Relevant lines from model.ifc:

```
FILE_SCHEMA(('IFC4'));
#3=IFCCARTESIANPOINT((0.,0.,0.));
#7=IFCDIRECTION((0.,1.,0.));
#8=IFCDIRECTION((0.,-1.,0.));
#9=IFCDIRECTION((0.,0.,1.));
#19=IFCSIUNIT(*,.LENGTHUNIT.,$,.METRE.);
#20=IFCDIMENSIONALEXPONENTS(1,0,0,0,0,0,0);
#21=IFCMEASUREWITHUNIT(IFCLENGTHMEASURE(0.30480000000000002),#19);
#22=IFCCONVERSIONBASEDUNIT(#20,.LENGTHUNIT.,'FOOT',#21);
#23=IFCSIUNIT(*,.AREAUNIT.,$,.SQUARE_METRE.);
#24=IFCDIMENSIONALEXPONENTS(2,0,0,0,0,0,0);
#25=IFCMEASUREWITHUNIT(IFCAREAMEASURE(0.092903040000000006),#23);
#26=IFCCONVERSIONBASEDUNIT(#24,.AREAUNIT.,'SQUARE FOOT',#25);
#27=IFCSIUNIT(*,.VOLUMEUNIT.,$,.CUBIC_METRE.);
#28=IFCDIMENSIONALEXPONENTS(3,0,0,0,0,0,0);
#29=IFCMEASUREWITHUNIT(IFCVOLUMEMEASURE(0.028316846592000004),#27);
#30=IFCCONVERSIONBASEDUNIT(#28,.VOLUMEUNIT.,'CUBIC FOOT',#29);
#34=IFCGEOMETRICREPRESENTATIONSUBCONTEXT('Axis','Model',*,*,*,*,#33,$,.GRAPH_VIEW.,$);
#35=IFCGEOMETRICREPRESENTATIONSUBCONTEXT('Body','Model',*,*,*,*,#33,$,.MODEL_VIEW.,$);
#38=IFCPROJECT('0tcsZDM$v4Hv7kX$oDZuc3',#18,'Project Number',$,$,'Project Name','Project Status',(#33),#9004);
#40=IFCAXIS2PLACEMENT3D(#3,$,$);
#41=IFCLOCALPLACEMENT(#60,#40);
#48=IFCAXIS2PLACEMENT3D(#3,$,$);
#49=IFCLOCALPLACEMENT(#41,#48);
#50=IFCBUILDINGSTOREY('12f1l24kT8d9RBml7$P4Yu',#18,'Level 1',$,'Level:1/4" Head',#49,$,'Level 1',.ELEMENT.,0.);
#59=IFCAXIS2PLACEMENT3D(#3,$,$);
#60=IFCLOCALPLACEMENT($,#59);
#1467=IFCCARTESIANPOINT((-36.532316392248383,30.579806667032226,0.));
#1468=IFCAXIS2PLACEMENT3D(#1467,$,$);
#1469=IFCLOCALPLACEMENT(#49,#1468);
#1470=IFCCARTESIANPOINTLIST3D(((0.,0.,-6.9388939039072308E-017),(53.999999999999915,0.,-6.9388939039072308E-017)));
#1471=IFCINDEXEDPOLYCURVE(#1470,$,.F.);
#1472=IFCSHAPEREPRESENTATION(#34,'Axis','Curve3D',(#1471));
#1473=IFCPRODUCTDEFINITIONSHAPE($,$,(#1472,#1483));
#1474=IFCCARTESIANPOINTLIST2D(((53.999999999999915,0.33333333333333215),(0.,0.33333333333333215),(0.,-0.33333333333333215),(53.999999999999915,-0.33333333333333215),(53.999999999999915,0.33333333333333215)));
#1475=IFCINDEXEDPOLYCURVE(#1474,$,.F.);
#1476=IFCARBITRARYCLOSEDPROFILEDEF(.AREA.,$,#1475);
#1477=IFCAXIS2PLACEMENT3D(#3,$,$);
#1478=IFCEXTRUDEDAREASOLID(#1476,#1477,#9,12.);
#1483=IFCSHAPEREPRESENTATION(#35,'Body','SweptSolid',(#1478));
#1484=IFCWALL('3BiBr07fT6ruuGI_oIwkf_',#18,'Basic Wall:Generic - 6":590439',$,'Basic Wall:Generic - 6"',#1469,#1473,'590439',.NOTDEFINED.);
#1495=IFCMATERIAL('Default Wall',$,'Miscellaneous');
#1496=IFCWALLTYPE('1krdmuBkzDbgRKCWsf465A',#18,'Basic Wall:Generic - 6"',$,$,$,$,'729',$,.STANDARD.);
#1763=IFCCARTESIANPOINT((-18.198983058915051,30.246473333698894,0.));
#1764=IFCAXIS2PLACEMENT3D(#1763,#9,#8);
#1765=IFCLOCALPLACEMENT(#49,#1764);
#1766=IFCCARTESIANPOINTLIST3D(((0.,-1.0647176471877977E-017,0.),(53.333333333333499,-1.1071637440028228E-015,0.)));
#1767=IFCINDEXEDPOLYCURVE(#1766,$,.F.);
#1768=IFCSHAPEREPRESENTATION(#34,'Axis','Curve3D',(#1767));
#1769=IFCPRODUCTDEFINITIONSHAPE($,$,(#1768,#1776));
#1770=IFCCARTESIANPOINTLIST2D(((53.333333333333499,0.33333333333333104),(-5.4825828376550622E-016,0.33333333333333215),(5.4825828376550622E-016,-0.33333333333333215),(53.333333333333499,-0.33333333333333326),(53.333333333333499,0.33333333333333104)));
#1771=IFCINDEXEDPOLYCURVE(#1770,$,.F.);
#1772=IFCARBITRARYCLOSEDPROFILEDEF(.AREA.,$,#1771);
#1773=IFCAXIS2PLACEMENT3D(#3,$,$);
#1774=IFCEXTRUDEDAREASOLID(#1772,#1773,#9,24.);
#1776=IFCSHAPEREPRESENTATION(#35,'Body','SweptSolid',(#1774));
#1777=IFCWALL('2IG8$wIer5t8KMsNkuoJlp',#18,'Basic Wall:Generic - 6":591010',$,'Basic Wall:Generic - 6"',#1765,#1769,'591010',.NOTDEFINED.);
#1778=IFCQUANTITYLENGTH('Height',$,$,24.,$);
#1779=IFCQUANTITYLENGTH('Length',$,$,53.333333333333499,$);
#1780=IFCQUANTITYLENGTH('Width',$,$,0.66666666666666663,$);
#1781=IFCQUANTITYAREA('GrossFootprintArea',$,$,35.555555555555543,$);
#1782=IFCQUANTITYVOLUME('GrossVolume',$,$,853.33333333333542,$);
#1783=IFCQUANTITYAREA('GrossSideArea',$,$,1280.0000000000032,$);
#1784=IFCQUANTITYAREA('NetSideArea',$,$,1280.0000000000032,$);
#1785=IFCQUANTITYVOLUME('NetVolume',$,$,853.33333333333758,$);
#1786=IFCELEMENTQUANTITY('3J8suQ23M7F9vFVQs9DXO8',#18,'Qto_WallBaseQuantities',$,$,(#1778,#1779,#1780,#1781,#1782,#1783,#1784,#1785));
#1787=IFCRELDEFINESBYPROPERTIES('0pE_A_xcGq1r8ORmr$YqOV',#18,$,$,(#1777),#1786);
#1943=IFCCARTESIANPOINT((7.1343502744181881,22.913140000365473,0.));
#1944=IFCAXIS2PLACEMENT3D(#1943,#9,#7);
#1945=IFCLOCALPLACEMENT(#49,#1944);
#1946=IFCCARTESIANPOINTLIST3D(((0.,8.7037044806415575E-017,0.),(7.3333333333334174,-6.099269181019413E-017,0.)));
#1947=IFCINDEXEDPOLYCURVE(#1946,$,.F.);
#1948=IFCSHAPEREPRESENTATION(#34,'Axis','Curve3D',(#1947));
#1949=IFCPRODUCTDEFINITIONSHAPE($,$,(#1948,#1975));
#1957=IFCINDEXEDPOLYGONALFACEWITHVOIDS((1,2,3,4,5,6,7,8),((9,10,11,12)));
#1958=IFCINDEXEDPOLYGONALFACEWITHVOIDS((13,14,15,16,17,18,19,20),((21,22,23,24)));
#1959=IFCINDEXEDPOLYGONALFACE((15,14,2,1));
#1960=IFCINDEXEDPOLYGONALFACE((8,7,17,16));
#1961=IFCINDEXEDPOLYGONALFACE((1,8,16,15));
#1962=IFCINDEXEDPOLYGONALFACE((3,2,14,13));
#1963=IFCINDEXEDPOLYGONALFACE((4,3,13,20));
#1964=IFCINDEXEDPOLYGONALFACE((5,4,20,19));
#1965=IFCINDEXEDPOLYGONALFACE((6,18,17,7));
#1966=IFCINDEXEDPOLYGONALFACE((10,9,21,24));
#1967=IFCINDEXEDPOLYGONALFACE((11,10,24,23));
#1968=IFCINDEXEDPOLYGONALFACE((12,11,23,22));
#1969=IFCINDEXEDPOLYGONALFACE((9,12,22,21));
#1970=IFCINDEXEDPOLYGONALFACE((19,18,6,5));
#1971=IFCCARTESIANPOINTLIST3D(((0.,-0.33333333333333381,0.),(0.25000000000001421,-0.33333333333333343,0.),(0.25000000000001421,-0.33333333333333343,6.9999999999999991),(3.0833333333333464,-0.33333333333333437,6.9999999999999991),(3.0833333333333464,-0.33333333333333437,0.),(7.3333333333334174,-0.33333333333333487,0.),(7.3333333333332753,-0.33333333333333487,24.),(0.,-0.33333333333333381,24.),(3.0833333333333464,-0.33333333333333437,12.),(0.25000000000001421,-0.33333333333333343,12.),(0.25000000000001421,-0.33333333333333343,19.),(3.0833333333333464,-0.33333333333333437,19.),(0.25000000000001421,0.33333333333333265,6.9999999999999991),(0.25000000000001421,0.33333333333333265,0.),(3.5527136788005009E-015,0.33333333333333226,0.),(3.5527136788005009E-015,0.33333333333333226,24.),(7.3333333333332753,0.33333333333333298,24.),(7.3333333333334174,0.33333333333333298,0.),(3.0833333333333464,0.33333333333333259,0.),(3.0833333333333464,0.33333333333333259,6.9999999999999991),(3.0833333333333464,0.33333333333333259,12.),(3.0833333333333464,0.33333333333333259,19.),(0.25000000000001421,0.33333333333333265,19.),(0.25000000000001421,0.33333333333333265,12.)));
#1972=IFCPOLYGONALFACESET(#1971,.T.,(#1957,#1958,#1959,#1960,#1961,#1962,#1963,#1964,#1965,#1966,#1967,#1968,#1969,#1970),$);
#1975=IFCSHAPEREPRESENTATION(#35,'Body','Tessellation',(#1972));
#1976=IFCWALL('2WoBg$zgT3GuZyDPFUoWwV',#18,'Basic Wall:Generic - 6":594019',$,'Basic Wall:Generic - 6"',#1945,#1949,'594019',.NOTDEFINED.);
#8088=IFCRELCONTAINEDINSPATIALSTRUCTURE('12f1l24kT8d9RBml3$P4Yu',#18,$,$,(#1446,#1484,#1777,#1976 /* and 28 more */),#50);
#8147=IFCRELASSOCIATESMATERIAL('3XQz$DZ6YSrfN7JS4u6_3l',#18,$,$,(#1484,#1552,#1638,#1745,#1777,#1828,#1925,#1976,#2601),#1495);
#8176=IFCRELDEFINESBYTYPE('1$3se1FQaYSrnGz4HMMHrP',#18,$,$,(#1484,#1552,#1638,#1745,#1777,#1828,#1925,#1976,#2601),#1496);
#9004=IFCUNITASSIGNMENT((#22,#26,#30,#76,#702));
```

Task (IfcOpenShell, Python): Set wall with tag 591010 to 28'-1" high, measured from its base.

```python
import ifcopenshell
import ifcopenshell.api.pset
import ifcopenshell.geom
import ifcopenshell.util.element
import ifcopenshell.util.representation
import ifcopenshell.util.shape
import ifcopenshell.util.unit

model = ifcopenshell.open("model.ifc")
unit_scale = ifcopenshell.util.unit.calculate_unit_scale(model)
area_scale = ifcopenshell.util.unit.calculate_unit_scale(model, "AREAUNIT")
volume_scale = ifcopenshell.util.unit.calculate_unit_scale(model, "VOLUMEUNIT")
settings = ifcopenshell.geom.settings()


def volume(element):
    """Net volume in cubic metres, openings subtracted."""
    shape = ifcopenshell.geom.create_shape(settings, element)
    return ifcopenshell.util.shape.get_volume(shape.geometry)


wall = model.by_guid("2IG8$wIer5t8KMsNkuoJlp")
before = volume(wall)

body = ifcopenshell.util.representation.get_representation(wall, "Model", "Body")
solid = body.Items[0]
old_height = solid.Depth
solid.Depth = 337 * 0.0254 / unit_scale
after = volume(wall)
thickness = 0.2032  # wall thickness in metres

# Update the stored height, areas and volumes.
qto = model.by_id(ifcopenshell.util.element.get_pset(wall, "Qto_WallBaseQuantities", should_inherit=False)["id"])
ifcopenshell.api.pset.edit_qto(model, qto=qto, properties={
    "Height": solid.Depth,
    "GrossVolume": ifcopenshell.util.element.get_pset(wall, "Qto_WallBaseQuantities", "GrossVolume") * solid.Depth / old_height,
    "GrossSideArea": ifcopenshell.util.element.get_pset(wall, "Qto_WallBaseQuantities", "GrossSideArea") * solid.Depth / old_height,
    "NetSideArea": after / thickness / area_scale,
    "NetVolume": after / volume_scale,
})

print(f"height {old_height:g} -> {solid.Depth:g}, volume {before:.3f} -> {after:.3f} m3")

model.write("model-out.ifc")
```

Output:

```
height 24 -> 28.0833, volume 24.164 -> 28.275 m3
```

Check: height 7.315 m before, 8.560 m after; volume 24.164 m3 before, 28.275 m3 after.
